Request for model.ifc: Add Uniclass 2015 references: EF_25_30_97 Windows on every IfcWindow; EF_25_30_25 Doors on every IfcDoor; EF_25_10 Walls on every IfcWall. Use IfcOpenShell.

First a look at what the model holds.

```python
import ifcopenshell

model = ifcopenshell.open("model.ifc")
print(model.schema)
print("classifications:", [c.Name for c in model.by_type("IfcClassification")])
for ifc_class in ("IfcDoor", "IfcRoof", "IfcStair", "IfcWall", "IfcWindow"):
    print(ifc_class, len(model.by_type(ifc_class)))
```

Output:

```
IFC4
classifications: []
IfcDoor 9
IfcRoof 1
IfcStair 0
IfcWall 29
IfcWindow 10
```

```python
import ifcopenshell
import ifcopenshell.api.classification

model = ifcopenshell.open("model.ifc")

system = ifcopenshell.api.classification.add_classification(model, classification="Uniclass 2015")

codes = {
    "IfcWindow": ("EF_25_30_97", "Windows"),
    "IfcDoor": ("EF_25_30_25", "Doors"),
    "IfcWall": ("EF_25_10", "Walls"),
}
for ifc_class, (code, name) in codes.items():
    products = model.by_type(ifc_class)
    ifcopenshell.api.classification.add_reference(
        model, products=products, classification=system, identification=code, name=name
    )
    print(code, len(products))

model.write("model_edited.ifc")
```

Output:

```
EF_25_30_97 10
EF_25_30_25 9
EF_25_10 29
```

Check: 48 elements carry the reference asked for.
